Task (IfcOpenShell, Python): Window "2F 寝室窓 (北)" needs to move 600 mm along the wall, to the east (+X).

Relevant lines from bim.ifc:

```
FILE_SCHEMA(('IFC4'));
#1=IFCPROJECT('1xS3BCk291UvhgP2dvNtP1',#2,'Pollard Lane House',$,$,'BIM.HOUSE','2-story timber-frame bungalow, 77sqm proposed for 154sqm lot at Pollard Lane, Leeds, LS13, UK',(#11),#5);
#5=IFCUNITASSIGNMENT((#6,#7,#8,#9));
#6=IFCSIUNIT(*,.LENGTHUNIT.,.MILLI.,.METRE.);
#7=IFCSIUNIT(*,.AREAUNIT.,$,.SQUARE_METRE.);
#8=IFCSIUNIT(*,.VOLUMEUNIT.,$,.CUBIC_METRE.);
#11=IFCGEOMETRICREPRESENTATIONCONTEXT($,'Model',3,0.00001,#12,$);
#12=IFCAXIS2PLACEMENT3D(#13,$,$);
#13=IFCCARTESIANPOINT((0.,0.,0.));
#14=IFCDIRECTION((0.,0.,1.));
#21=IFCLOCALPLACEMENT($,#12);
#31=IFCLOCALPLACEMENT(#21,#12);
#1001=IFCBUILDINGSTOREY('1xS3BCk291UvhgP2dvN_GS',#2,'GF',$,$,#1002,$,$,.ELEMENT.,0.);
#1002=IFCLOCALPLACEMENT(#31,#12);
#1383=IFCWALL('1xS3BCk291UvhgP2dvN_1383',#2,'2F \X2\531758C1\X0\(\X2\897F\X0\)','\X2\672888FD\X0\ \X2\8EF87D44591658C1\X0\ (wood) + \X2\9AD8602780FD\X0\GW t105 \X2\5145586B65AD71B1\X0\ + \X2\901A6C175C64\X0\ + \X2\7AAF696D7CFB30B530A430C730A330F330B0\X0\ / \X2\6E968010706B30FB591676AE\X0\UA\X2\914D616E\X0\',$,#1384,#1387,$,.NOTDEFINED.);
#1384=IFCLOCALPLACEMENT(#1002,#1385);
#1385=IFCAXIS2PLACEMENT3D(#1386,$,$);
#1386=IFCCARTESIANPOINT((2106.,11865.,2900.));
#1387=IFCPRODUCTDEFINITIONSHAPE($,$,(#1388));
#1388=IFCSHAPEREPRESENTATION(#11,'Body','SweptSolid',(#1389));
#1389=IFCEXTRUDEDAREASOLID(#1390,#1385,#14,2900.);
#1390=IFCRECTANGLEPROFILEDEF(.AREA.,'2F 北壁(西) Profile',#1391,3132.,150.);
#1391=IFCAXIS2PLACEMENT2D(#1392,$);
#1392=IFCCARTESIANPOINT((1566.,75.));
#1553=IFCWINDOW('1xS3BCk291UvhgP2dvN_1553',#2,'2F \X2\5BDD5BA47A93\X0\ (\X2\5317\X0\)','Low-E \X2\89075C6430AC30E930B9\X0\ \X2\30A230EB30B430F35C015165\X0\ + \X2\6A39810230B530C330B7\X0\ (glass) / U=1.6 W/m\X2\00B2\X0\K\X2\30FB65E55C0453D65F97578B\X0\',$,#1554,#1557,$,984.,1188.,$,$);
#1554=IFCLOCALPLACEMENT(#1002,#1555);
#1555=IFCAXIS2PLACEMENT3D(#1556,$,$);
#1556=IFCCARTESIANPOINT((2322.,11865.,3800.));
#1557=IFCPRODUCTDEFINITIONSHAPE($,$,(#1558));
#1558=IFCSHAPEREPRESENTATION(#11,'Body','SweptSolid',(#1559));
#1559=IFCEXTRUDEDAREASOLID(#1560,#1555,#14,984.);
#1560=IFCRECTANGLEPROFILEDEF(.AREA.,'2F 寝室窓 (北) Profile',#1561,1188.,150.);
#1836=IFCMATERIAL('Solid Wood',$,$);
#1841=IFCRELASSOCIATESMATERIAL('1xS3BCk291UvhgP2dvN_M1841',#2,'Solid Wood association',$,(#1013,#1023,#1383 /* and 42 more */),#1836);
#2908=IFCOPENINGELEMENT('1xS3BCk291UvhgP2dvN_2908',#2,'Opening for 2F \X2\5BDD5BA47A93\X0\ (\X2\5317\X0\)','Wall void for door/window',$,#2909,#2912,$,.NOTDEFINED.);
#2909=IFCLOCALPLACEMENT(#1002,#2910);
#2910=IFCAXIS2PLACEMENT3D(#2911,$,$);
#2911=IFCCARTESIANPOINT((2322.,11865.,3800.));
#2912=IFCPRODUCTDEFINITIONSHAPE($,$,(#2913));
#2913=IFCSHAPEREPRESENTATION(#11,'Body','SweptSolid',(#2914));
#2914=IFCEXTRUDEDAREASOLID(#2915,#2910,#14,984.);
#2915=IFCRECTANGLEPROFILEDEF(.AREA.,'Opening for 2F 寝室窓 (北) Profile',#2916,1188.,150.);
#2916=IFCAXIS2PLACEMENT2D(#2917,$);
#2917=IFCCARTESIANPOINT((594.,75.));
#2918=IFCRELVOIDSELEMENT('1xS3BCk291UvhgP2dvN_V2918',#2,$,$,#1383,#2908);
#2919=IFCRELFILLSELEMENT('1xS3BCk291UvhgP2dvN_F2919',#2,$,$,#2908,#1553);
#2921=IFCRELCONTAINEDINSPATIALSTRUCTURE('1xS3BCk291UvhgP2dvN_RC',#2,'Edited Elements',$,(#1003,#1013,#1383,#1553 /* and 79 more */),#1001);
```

```python
import ifcopenshell
import ifcopenshell.api.geometry
import ifcopenshell.util.placement
import ifcopenshell.util.unit

model = ifcopenshell.open("bim.ifc")
unit_scale = ifcopenshell.util.unit.calculate_unit_scale(model)

window = model.by_id(1553)
opening = window.FillsVoids[0].RelatingOpeningElement
wall = opening.VoidsElements[0].RelatingBuildingElement

wall_matrix = ifcopenshell.util.placement.get_local_placement(wall.ObjectPlacement)
shift = wall_matrix[:3, 0] * 0.6 / unit_scale
before = ifcopenshell.util.placement.get_local_placement(window.ObjectPlacement)[:3, 3].copy()

# The window is not placed relative to its opening, so move both.
for product in (opening, window):
    matrix = ifcopenshell.util.placement.get_local_placement(product.ObjectPlacement)
    matrix[:3, 3] += shift
    ifcopenshell.api.geometry.edit_object_placement(model, product=product, matrix=matrix, is_si=False)

after = ifcopenshell.util.placement.get_local_placement(window.ObjectPlacement)[:3, 3]
print("window moved by", (after - before).round(3) + 0.0)

model.write("bim-out.ifc")
```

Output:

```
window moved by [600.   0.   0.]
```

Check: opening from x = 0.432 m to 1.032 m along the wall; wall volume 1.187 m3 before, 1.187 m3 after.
